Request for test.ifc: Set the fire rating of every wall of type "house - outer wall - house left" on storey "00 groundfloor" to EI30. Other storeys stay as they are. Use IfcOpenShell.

First a look at what the model holds.

```python
import ifcopenshell
import ifcopenshell.util.element

model = ifcopenshell.open("test.ifc")
print(model.schema)
storey = next(s for s in model.by_type("IfcBuildingStorey") if s.Name == "00 groundfloor")
walls = [e for e in ifcopenshell.util.element.get_decomposition(storey) if e.is_a("IfcWall")]
seen = {}
for e in walls:
    element_type = ifcopenshell.util.element.get_type(e)
    key = (element_type.Name if element_type != e and element_type else None, ifcopenshell.util.element.get_pset(e, "Pset_WallCommon", "FireRating"))
    seen[key] = seen.get(key, 0) + 1
for (name, value), count in sorted(seen.items(), key=str):
    print(count, "x", name, "|", value)
```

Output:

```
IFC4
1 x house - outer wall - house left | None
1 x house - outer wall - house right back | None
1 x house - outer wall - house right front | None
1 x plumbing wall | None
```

```python
import ifcopenshell
import ifcopenshell.api.pset
import ifcopenshell.util.element

model = ifcopenshell.open("test.ifc")

storey = next(s for s in model.by_type("IfcBuildingStorey") if s.Name == "00 groundfloor")
walls = [e for e in ifcopenshell.util.element.get_decomposition(storey) if e.is_a("IfcWall")]

count = 0
for e in walls:
    element_type = ifcopenshell.util.element.get_type(e)
    if element_type in (None, e) or element_type.Name != "house - outer wall - house left":
        continue
    # add_pset returns the element's existing set when there is one.
    pset = ifcopenshell.api.pset.add_pset(model, product=e, name="Pset_WallCommon")
    ifcopenshell.api.pset.edit_pset(model, pset=pset, properties={"FireRating": "EI30"})
    count += 1

print(count, "walls updated")

model.write("test_updated.ifc")
```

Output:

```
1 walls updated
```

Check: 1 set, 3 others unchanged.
